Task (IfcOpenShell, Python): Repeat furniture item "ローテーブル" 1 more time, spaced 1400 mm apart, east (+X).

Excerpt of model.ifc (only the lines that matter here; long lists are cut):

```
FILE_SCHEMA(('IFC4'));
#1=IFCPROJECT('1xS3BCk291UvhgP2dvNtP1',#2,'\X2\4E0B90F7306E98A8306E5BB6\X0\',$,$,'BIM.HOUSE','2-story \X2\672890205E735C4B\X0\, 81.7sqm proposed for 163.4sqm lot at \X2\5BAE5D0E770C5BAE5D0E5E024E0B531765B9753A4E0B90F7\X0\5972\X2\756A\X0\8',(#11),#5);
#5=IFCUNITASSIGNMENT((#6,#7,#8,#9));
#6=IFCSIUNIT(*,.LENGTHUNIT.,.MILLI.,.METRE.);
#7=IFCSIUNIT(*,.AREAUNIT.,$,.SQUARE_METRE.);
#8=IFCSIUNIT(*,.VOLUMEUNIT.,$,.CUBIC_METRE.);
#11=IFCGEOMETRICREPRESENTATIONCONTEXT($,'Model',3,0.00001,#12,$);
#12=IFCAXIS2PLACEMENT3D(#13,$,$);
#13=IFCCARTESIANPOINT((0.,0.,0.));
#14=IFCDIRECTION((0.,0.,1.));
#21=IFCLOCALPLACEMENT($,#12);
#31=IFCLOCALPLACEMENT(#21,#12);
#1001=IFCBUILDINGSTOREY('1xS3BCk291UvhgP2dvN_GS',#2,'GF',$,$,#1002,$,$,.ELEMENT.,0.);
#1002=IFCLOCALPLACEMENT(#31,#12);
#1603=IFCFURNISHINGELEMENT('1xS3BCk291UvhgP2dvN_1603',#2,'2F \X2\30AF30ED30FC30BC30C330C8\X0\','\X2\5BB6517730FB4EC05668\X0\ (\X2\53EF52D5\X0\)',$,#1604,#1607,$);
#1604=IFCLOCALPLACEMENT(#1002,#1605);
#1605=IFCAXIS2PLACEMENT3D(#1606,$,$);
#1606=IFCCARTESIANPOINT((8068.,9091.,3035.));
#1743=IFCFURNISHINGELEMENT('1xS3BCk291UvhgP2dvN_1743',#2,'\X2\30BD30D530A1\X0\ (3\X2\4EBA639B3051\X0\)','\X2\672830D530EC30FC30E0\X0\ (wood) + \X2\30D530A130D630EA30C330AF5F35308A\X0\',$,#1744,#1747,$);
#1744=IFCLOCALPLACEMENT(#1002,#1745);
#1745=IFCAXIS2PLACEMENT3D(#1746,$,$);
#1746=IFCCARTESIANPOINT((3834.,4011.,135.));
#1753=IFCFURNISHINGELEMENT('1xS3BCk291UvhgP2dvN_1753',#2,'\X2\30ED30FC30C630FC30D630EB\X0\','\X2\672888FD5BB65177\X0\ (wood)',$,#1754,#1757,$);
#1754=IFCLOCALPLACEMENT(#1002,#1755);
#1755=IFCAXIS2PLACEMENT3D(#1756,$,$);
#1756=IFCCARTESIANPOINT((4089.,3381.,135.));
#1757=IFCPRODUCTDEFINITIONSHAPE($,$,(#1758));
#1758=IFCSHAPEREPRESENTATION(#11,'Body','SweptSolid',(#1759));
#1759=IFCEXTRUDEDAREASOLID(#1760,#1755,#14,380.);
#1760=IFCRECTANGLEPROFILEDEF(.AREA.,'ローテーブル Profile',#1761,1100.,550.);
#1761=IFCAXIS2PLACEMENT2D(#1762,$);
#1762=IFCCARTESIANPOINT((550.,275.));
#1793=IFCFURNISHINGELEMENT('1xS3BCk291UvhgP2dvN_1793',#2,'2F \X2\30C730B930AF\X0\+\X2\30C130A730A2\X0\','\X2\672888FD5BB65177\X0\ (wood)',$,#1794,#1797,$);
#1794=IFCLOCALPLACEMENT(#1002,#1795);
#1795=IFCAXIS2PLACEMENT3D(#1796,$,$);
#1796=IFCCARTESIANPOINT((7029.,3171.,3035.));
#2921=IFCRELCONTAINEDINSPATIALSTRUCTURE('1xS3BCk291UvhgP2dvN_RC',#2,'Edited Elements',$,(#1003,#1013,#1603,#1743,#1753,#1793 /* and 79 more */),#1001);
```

```python
import numpy as np
import ifcopenshell
import ifcopenshell.api.geometry
import ifcopenshell.api.root
import ifcopenshell.util.element
import ifcopenshell.util.placement
import ifcopenshell.util.unit

model = ifcopenshell.open("model.ifc")
unit_scale = ifcopenshell.util.unit.calculate_unit_scale(model)


def reuse_history(source, copy):
    """copy_class also copies each property set's owner history, people and application; keep the originals."""
    for rel in copy.IsDefinedBy:
        if rel.is_a("IfcRelDefinesByProperties") and (history := rel.RelatingPropertyDefinition.OwnerHistory):
            rel.RelatingPropertyDefinition.OwnerHistory = source.OwnerHistory
            ifcopenshell.util.element.remove_deep2(model, history)


source = model.by_id(1753)
base = ifcopenshell.util.placement.get_local_placement(source.ObjectPlacement)
step = np.array([1.0, 0.0, 0.0]) * 1.4 / unit_scale

for i in range(1, 2):
    copy = ifcopenshell.api.root.copy_class(model, product=source)
    copy.Representation = ifcopenshell.util.element.copy_deep(
        model, source.Representation, exclude=["IfcGeometricRepresentationContext", "IfcRepresentationMap"]
    )
    reuse_history(source, copy)
    matrix = base.copy()
    matrix[:3, 3] += i * step
    print("added at", matrix[:3, 3].round(3) + 0.0)
    ifcopenshell.api.geometry.edit_object_placement(model, product=copy, matrix=matrix, is_si=False)

model.write("model-out.ifc")
```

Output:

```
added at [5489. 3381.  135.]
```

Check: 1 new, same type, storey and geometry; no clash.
